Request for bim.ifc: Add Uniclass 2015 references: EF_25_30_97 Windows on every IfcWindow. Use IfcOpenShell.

First a look at what the model holds.

```python
import ifcopenshell

model = ifcopenshell.open("bim.ifc")
print(model.schema)
print("classifications:", [c.Name for c in model.by_type("IfcClassification")])
for ifc_class in ("IfcDoor", "IfcRoof", "IfcStair", "IfcWall", "IfcWindow"):
    print(ifc_class, len(model.by_type(ifc_class)))
```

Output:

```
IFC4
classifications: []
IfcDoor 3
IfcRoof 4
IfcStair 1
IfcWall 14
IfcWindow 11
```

```python
import ifcopenshell
import ifcopenshell.api.classification

model = ifcopenshell.open("bim.ifc")

system = ifcopenshell.api.classification.add_classification(model, classification="Uniclass 2015")

codes = {
    "IfcWindow": ("EF_25_30_97", "Windows"),
}
for ifc_class, (code, name) in codes.items():
    products = model.by_type(ifc_class)
    ifcopenshell.api.classification.add_reference(
        model, products=products, classification=system, identification=code, name=name
    )
    print(code, len(products))

model.write("bim_v2.ifc")
```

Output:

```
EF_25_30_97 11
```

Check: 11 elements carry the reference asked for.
